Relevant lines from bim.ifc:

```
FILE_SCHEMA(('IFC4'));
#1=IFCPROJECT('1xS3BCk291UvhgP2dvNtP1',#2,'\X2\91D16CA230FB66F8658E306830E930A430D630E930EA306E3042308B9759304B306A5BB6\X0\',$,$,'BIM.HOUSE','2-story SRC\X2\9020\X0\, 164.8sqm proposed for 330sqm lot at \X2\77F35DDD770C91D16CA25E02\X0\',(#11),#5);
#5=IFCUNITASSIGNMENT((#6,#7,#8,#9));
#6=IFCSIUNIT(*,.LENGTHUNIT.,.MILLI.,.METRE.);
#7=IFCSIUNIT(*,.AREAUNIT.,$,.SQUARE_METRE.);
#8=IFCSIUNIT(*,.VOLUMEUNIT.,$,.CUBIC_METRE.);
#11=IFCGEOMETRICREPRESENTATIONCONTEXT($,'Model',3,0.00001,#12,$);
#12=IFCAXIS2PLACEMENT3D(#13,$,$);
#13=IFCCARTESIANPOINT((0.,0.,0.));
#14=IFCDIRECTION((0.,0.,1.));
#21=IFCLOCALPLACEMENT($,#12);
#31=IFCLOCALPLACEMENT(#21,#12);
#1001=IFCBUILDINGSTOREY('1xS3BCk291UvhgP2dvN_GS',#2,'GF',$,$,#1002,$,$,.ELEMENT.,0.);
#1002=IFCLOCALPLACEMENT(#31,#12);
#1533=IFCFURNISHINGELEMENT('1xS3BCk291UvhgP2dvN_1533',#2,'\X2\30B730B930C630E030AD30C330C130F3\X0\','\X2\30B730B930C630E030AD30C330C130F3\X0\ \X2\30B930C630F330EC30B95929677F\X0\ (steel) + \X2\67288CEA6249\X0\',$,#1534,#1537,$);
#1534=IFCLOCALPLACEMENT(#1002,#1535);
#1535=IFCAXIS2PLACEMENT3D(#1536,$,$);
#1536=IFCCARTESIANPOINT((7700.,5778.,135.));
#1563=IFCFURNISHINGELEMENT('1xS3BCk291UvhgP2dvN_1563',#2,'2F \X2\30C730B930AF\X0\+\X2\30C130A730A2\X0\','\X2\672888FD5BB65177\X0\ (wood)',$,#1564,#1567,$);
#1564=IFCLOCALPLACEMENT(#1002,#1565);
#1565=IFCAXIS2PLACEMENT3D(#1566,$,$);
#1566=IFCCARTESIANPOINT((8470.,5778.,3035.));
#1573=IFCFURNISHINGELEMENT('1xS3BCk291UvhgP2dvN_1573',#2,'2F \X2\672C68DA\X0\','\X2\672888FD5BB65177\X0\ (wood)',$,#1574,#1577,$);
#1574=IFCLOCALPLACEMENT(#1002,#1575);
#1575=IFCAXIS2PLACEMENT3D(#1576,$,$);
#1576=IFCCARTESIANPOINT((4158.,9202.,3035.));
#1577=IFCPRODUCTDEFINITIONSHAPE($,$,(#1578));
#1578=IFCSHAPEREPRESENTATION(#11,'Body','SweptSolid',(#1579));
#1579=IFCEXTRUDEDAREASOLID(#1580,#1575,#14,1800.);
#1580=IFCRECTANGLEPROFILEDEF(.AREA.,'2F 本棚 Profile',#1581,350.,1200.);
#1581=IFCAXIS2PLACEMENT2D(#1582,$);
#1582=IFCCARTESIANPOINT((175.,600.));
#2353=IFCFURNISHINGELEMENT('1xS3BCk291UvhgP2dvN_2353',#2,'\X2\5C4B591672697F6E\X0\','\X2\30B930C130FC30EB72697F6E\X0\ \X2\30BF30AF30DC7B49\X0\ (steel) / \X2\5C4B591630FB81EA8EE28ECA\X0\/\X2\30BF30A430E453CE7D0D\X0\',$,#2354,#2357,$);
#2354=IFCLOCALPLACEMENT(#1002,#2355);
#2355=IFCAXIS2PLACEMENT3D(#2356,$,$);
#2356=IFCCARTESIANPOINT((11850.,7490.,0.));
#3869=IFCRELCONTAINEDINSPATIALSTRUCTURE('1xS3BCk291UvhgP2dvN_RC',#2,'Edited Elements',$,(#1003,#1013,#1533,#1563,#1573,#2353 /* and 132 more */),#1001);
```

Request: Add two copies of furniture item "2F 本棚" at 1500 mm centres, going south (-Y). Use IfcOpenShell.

```python
import numpy as np
import ifcopenshell
import ifcopenshell.api.geometry
import ifcopenshell.api.root
import ifcopenshell.util.element
import ifcopenshell.util.placement

model = ifcopenshell.open("bim.ifc")


def reuse_history(source, copy):
    """copy_class also copies each property set's owner history, people and application; keep the originals."""
    for rel in copy.IsDefinedBy:
        if rel.is_a("IfcRelDefinesByProperties") and (history := rel.RelatingPropertyDefinition.OwnerHistory):
            rel.RelatingPropertyDefinition.OwnerHistory = source.OwnerHistory
            ifcopenshell.util.element.remove_deep2(model, history)


source = model.by_id(1573)
base = ifcopenshell.util.placement.get_local_placement(source.ObjectPlacement)
step = np.array([0.0, -1.0, 0.0]) * 1500.0

for i in range(1, 3):
    copy = ifcopenshell.api.root.copy_class(model, product=source)
    copy.Representation = ifcopenshell.util.element.copy_deep(
        model, source.Representation, exclude=["IfcGeometricRepresentationContext", "IfcRepresentationMap"]
    )
    reuse_history(source, copy)
    matrix = base.copy()
    matrix[:3, 3] += i * step
    print("added at", matrix[:3, 3].round(3) + 0.0)
    ifcopenshell.api.geometry.edit_object_placement(model, product=copy, matrix=matrix, is_si=False)

model.write("bim_edited.ifc")
```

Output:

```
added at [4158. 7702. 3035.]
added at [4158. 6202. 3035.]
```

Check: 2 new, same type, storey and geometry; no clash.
